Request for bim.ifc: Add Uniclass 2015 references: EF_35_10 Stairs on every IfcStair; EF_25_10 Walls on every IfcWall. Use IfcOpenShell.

First a look at what the model holds.

```python
import ifcopenshell

model = ifcopenshell.open("bim.ifc")
print(model.schema)
print("classifications:", [c.Name for c in model.by_type("IfcClassification")])
for ifc_class in ("IfcDoor", "IfcRoof", "IfcStair", "IfcWall", "IfcWindow"):
    print(ifc_class, len(model.by_type(ifc_class)))
```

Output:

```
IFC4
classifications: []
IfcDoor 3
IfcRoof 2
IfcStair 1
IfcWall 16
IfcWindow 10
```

```python
import ifcopenshell
import ifcopenshell.api.classification

model = ifcopenshell.open("bim.ifc")

system = ifcopenshell.api.classification.add_classification(model, classification="Uniclass 2015")

codes = {
    "IfcStair": ("EF_35_10", "Stairs"),
    "IfcWall": ("EF_25_10", "Walls"),
}
for ifc_class, (code, name) in codes.items():
    products = model.by_type(ifc_class)
    ifcopenshell.api.classification.add_reference(
        model, products=products, classification=system, identification=code, name=name
    )
    print(code, len(products))

model.write("bim_updated.ifc")
```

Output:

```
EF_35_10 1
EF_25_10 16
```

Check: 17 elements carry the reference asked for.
